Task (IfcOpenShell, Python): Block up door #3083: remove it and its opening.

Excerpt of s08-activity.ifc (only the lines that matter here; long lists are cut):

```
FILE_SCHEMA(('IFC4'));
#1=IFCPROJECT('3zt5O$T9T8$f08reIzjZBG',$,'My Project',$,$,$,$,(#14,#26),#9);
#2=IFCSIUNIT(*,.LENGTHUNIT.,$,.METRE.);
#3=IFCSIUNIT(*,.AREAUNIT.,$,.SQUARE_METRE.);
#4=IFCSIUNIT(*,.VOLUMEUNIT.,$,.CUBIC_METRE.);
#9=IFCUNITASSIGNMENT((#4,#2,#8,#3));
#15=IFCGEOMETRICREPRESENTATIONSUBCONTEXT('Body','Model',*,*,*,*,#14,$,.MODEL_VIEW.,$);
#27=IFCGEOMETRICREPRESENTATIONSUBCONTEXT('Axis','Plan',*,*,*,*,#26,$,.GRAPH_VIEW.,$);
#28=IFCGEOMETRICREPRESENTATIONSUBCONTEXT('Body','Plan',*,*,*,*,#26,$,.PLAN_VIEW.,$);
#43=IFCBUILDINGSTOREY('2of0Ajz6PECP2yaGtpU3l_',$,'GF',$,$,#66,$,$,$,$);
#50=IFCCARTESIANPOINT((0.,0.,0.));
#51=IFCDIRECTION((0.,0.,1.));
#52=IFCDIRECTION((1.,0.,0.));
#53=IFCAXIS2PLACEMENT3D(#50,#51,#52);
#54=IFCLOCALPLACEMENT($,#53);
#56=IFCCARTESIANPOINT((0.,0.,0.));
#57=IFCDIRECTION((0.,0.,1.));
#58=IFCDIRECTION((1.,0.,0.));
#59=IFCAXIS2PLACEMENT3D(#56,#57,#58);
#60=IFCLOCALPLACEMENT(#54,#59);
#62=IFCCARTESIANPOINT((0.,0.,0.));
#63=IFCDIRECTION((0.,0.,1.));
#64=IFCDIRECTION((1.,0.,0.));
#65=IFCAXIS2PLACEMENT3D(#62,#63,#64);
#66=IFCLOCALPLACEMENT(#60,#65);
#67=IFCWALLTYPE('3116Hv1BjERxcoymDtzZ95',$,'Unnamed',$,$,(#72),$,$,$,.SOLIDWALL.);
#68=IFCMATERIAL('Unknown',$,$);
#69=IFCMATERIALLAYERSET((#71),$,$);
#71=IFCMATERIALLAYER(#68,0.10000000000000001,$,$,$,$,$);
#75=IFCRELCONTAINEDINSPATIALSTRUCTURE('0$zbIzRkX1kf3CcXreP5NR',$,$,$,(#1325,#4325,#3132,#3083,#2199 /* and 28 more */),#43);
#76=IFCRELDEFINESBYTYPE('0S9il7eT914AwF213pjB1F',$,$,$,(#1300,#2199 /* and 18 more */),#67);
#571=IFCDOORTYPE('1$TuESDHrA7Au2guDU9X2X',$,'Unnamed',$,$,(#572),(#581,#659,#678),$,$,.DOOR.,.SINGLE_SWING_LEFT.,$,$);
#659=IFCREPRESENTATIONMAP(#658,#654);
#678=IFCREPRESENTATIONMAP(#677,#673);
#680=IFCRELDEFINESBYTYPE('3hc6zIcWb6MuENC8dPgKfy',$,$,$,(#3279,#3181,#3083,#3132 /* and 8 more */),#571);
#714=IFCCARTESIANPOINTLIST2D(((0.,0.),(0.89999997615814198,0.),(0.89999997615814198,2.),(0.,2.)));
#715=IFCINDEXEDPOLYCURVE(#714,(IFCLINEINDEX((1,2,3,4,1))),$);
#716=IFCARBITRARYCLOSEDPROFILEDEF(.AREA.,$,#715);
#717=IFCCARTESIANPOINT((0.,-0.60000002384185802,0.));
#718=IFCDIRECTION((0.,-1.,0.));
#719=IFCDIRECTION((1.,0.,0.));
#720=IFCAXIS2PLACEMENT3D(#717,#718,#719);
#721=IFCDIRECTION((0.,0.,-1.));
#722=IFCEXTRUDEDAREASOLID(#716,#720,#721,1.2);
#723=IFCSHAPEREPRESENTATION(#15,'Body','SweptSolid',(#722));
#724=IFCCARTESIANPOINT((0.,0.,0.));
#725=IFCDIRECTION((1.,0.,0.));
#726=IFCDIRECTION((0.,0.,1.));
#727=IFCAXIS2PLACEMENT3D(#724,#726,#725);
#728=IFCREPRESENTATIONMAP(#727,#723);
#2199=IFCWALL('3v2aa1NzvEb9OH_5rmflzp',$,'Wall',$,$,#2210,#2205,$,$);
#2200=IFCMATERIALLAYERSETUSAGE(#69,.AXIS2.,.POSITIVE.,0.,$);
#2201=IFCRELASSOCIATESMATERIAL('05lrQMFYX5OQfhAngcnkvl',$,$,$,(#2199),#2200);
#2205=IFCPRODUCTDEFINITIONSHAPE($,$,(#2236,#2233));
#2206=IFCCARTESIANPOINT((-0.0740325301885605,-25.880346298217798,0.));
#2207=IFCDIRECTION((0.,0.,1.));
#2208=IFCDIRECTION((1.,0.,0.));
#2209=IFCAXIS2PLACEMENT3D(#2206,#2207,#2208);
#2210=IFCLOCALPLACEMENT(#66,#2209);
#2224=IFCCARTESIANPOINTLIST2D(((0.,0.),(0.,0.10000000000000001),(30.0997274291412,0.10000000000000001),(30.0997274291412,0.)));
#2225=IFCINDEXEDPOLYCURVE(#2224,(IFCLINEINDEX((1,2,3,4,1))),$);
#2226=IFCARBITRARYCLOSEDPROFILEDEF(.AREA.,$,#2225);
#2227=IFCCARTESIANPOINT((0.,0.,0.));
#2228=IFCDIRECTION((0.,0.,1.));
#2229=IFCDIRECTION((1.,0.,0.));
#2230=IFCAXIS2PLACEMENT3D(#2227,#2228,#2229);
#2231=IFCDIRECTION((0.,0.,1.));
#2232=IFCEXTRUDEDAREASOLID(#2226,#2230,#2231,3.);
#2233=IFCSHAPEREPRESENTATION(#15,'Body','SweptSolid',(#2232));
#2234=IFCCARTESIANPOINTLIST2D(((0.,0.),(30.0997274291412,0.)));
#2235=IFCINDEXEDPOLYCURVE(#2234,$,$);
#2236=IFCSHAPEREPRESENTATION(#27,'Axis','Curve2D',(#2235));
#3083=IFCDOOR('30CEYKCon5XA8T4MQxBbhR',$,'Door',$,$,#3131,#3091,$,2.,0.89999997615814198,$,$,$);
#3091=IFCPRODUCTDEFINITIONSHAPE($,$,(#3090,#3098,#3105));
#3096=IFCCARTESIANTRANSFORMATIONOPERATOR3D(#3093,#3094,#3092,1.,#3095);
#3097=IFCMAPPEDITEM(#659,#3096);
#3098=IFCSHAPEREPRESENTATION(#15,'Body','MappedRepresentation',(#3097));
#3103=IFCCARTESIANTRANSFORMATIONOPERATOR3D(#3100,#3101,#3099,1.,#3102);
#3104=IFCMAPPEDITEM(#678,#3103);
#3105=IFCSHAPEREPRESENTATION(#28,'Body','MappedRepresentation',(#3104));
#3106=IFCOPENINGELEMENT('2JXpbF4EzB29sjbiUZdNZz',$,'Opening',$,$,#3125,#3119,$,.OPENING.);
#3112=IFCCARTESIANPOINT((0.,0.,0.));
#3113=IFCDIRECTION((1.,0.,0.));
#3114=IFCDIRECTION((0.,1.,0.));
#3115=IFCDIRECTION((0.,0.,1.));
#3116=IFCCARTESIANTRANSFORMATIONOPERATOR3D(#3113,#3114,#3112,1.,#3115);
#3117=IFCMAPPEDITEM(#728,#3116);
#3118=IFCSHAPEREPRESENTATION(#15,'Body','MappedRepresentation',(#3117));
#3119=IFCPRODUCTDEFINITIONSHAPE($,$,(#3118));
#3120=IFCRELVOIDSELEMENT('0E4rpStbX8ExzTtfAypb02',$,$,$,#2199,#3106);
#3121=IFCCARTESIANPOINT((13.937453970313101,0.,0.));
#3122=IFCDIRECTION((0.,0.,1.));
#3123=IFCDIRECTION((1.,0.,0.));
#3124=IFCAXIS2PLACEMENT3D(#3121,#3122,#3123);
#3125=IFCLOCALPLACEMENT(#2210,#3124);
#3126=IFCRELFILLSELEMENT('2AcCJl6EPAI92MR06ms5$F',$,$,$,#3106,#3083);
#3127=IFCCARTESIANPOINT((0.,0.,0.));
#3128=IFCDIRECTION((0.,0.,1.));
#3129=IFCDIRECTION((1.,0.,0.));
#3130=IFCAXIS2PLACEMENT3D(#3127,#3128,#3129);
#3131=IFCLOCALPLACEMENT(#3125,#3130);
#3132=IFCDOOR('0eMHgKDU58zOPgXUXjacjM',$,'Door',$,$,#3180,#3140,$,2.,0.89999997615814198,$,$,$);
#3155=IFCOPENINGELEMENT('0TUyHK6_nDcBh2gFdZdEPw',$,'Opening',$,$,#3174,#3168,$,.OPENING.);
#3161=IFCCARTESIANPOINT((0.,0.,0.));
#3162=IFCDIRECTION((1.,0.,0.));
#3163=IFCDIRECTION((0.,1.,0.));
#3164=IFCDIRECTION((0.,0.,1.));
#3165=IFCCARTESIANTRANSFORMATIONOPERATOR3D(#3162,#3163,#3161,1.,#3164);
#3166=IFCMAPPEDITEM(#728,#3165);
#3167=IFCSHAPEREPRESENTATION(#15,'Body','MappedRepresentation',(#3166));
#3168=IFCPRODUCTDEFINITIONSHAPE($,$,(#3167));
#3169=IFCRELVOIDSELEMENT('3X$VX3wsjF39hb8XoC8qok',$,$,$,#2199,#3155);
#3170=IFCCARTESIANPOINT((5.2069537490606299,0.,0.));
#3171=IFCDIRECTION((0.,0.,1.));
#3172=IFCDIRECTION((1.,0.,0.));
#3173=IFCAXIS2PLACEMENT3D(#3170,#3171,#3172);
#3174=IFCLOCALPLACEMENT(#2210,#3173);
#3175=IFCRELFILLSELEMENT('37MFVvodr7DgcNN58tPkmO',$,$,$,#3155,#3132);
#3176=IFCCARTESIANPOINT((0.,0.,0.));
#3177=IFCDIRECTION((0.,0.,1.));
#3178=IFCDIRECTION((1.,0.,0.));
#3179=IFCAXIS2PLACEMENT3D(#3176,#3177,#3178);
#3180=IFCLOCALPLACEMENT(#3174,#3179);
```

```python
import ifcopenshell
import ifcopenshell.api.feature
import ifcopenshell.api.root
import ifcopenshell.geom
import ifcopenshell.util.shape

model = ifcopenshell.open("s08-activity.ifc")
settings = ifcopenshell.geom.settings()


def volume(element):
    """Net volume in cubic metres, openings subtracted."""
    shape = ifcopenshell.geom.create_shape(settings, element)
    return ifcopenshell.util.shape.get_volume(shape.geometry)


door = model.by_guid("30CEYKCon5XA8T4MQxBbhR")
opening = door.FillsVoids[0].RelatingOpeningElement
wall = opening.VoidsElements[0].RelatingBuildingElement
before = volume(wall)

ifcopenshell.api.root.remove_product(model, product=door)
ifcopenshell.api.feature.remove_feature(model, feature=opening)

after = volume(wall)

print(f"wall volume {before:.3f} -> {after:.3f} m3")

model.write("s08-activity_edited.ifc")
```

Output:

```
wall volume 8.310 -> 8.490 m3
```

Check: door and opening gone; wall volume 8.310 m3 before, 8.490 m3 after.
